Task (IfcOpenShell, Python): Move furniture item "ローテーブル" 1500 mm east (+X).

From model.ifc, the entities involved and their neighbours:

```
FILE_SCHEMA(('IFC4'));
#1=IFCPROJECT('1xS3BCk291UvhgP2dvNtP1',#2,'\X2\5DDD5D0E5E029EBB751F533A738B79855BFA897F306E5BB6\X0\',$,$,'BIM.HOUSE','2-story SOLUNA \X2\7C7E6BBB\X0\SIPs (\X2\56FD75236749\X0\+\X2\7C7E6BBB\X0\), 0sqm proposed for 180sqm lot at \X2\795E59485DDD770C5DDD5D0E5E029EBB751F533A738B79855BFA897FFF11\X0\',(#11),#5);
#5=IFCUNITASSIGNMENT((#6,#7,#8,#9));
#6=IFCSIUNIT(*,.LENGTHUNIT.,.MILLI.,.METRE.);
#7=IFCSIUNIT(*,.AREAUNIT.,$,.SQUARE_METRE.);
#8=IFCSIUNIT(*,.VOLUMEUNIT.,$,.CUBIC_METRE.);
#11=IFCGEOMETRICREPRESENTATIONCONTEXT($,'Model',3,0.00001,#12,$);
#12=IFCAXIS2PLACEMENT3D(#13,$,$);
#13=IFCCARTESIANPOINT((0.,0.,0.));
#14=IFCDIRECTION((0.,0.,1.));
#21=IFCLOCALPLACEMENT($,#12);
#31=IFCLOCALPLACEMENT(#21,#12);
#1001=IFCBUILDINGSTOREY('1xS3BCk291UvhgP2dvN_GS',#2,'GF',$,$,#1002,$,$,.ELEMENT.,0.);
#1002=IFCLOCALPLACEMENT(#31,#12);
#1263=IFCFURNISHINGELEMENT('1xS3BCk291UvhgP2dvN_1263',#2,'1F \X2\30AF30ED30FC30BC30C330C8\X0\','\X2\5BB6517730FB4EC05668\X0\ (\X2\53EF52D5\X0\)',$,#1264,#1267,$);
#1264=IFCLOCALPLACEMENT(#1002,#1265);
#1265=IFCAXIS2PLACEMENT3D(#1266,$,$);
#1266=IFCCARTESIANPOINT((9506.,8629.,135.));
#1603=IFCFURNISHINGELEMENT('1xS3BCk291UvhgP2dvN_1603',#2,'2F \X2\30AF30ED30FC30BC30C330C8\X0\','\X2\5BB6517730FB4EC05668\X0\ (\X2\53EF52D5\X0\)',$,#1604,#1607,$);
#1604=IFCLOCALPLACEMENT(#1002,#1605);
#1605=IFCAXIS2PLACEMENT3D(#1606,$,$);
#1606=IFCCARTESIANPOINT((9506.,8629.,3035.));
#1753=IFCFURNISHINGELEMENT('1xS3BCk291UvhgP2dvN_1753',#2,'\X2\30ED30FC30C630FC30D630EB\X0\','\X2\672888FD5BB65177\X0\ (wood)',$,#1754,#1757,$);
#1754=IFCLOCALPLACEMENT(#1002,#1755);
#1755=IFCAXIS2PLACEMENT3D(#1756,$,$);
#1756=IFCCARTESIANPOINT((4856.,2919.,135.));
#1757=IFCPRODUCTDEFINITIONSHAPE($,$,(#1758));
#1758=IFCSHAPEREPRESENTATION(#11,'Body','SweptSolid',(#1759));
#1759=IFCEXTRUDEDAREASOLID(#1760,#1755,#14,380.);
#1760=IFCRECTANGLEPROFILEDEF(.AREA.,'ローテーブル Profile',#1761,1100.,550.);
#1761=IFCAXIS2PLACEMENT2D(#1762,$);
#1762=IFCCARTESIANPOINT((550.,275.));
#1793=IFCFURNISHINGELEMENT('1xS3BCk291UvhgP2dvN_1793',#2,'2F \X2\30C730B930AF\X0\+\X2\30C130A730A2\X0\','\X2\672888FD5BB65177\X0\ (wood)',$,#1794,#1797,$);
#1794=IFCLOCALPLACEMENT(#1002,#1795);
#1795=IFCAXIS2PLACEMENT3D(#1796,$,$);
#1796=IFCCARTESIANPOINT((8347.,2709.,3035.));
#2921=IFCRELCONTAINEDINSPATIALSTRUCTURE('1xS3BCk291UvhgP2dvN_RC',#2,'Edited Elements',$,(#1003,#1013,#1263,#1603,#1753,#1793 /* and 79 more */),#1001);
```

```python
import ifcopenshell
import ifcopenshell.api.geometry
import ifcopenshell.util.placement
import ifcopenshell.util.unit

model = ifcopenshell.open("model.ifc")
unit_scale = ifcopenshell.util.unit.calculate_unit_scale(model)

item = model.by_guid("1xS3BCk291UvhgP2dvN_1753")
matrix = ifcopenshell.util.placement.get_local_placement(item.ObjectPlacement)
matrix[0, 3] += 1.5 / unit_scale
ifcopenshell.api.geometry.edit_object_placement(model, product=item, matrix=matrix, is_si=False)

print(ifcopenshell.util.placement.get_local_placement(item.ObjectPlacement).round(3) + 0.0)

model.write("model-out.ifc")
```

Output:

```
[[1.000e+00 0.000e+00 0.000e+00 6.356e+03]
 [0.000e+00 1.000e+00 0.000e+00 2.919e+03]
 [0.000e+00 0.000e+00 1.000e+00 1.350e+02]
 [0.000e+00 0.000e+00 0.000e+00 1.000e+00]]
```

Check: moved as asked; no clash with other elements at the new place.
